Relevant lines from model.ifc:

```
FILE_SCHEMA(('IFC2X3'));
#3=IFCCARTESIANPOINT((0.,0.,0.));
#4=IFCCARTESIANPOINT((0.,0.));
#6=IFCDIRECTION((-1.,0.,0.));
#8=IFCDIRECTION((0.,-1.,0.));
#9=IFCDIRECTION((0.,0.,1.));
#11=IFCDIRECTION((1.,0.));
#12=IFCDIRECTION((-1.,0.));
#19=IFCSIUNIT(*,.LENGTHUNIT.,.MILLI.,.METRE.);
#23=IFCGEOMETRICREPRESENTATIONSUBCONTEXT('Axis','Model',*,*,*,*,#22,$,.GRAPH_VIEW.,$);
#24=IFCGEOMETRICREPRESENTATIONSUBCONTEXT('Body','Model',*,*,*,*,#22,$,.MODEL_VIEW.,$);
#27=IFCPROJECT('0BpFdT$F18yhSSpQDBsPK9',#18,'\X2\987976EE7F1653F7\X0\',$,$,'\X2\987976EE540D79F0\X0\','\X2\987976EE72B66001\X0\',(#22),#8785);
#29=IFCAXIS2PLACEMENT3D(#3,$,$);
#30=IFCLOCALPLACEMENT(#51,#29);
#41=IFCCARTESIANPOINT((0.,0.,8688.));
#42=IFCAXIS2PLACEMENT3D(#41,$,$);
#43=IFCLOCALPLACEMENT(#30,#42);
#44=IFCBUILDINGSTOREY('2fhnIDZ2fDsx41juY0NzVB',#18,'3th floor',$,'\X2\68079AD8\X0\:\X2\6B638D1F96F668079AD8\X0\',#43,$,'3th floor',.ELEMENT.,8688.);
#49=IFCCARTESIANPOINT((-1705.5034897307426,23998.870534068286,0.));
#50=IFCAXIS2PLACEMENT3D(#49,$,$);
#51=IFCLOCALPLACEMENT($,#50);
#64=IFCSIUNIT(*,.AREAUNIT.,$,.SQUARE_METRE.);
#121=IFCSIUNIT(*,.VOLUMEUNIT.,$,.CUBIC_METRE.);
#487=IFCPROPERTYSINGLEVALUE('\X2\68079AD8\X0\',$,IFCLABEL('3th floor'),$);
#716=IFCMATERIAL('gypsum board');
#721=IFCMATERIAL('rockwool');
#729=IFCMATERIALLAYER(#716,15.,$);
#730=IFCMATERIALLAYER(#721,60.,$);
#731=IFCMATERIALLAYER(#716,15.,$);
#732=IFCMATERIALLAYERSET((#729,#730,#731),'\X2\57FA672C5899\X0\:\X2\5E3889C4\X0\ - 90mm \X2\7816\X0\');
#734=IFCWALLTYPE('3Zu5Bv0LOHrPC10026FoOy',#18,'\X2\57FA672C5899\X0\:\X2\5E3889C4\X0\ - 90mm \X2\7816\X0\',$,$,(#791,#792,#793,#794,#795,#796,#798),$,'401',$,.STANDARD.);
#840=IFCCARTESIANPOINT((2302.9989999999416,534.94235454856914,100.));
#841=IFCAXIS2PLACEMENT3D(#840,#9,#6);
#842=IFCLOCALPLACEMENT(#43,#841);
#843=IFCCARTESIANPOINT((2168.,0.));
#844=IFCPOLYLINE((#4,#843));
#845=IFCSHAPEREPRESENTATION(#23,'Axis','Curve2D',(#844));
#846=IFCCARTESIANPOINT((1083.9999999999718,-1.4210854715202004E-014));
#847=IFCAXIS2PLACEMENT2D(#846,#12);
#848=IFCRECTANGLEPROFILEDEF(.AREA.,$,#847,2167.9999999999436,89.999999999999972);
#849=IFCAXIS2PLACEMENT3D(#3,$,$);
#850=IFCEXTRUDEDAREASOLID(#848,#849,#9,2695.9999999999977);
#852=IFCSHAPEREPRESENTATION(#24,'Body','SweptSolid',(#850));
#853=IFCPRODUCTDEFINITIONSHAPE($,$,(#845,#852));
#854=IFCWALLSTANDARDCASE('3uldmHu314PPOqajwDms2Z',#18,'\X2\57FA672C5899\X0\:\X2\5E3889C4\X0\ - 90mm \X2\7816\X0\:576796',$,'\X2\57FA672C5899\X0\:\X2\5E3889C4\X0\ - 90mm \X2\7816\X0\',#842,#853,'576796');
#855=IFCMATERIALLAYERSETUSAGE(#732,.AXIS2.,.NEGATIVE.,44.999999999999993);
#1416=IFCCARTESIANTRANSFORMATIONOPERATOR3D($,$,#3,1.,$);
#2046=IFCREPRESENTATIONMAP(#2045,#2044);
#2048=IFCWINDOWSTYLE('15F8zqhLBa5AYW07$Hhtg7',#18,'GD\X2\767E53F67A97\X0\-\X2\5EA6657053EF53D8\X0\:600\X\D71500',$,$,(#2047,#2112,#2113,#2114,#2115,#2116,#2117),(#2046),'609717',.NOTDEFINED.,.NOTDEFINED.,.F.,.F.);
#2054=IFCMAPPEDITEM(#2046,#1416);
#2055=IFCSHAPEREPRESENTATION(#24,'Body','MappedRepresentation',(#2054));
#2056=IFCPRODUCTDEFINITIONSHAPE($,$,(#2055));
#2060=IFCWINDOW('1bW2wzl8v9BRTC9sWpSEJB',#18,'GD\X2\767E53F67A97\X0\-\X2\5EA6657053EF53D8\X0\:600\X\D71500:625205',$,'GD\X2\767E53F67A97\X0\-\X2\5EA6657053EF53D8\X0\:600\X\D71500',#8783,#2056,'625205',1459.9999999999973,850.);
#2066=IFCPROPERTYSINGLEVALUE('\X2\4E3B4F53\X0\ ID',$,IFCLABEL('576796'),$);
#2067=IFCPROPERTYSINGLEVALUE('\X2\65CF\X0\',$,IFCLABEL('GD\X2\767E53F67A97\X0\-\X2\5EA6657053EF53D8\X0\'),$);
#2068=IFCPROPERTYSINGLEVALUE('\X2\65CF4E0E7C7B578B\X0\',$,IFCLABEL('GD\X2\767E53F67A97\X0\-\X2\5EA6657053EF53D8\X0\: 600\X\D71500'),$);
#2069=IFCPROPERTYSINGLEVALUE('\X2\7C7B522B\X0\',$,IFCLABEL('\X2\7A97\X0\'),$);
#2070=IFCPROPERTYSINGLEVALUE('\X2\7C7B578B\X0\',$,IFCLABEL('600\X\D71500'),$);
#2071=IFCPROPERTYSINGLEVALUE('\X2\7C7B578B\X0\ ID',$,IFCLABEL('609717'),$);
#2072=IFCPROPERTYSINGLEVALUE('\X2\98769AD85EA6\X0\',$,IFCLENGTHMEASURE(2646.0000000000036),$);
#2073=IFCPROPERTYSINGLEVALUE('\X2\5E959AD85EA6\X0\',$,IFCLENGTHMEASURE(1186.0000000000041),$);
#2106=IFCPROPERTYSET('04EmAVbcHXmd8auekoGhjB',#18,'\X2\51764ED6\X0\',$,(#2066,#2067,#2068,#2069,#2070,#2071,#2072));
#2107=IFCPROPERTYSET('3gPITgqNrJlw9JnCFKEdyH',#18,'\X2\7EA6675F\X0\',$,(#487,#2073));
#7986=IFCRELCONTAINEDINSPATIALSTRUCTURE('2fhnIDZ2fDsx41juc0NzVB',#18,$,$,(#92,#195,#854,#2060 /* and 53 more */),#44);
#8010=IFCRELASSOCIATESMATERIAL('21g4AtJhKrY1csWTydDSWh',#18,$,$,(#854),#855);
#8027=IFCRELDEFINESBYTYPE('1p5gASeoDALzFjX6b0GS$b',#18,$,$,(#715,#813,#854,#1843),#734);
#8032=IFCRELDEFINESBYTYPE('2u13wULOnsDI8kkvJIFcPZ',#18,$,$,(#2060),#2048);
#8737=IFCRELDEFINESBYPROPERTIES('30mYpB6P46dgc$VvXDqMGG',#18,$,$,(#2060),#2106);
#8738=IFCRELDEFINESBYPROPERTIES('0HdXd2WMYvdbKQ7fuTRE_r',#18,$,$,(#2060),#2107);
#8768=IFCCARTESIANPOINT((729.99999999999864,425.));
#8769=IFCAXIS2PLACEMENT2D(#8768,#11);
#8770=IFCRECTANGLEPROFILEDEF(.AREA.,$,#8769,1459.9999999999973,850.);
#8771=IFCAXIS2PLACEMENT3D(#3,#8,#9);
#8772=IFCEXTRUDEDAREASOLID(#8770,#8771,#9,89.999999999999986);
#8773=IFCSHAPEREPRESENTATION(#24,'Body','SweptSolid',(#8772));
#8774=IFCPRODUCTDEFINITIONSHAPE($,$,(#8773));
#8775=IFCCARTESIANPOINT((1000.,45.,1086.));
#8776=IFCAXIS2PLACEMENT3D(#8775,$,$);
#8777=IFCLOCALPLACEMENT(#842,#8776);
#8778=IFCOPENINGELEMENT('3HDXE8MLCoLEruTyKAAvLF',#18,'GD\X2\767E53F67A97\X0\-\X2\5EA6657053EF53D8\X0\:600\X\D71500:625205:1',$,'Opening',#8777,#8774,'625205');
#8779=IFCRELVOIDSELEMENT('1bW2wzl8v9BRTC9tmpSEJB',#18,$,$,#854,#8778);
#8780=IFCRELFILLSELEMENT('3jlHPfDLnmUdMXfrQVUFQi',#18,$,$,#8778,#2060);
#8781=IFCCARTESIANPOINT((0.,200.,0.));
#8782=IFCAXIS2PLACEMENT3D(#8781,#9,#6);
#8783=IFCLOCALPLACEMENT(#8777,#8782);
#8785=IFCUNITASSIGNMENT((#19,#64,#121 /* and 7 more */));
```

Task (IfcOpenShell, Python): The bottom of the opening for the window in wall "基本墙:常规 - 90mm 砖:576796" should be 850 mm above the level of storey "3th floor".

```python
import numpy as np
import ifcopenshell
import ifcopenshell.api.geometry
import ifcopenshell.api.pset
import ifcopenshell.geom
import ifcopenshell.util.element
import ifcopenshell.util.placement
import ifcopenshell.util.shape
import ifcopenshell.util.unit

model = ifcopenshell.open("model.ifc")
unit_scale = ifcopenshell.util.unit.calculate_unit_scale(model)

window = model.by_guid("1bW2wzl8v9BRTC9sWpSEJB")
opening = window.FillsVoids[0].RelatingOpeningElement
storey = ifcopenshell.util.element.get_container(window, ifc_class="IfcBuildingStorey")
level = ifcopenshell.util.placement.get_local_placement(storey.ObjectPlacement)[2, 3]

# The opening's origin need not be at the sill, so measure its lowest point.
shape = ifcopenshell.geom.create_shape(ifcopenshell.geom.settings(), opening)
bottom = ifcopenshell.util.shape.get_shape_bottom_elevation(shape, shape.geometry) / unit_scale
dz = level + 850.0 - bottom

shift = np.array([0.0, 0.0, dz])
# The window is placed relative to its opening, so it follows when the opening moves.
matrix = ifcopenshell.util.placement.get_local_placement(opening.ObjectPlacement)
matrix[:3, 3] += shift
ifcopenshell.api.geometry.edit_object_placement(
    model, product=opening, matrix=matrix, is_si=False, should_transform_children=True
)

# Keep the stored heights in step.
pset = model.by_id(ifcopenshell.util.element.get_pset(window, "其他", should_inherit=False)["id"])
ifcopenshell.api.pset.edit_pset(model, pset=pset, properties={
    "顶高度": model.create_entity("IfcLengthMeasure", ifcopenshell.util.element.get_pset(window, "其他", "顶高度") + dz),
})
pset = model.by_id(ifcopenshell.util.element.get_pset(window, "约束", should_inherit=False)["id"])
ifcopenshell.api.pset.edit_pset(model, pset=pset, properties={
    "底高度": model.create_entity("IfcLengthMeasure", ifcopenshell.util.element.get_pset(window, "约束", "底高度") + dz),
})

print(f"moved by {dz * unit_scale:+.3f} m")

model.write("model_updated.ifc")
```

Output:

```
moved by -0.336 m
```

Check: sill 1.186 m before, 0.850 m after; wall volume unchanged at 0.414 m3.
